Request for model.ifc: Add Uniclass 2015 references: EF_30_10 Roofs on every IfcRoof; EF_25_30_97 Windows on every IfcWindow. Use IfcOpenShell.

First a look at what the model holds.

```python
import ifcopenshell

model = ifcopenshell.open("model.ifc")
print(model.schema)
print("classifications:", [c.Name for c in model.by_type("IfcClassification")])
for ifc_class in ("IfcDoor", "IfcRoof", "IfcStair", "IfcWall", "IfcWindow"):
    print(ifc_class, len(model.by_type(ifc_class)))
```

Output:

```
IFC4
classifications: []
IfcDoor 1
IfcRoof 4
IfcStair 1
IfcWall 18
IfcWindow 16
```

```python
import ifcopenshell
import ifcopenshell.api.classification

model = ifcopenshell.open("model.ifc")

system = ifcopenshell.api.classification.add_classification(model, classification="Uniclass 2015")

codes = {
    "IfcRoof": ("EF_30_10", "Roofs"),
    "IfcWindow": ("EF_25_30_97", "Windows"),
}
for ifc_class, (code, name) in codes.items():
    products = model.by_type(ifc_class)
    ifcopenshell.api.classification.add_reference(
        model, products=products, classification=system, identification=code, name=name
    )
    print(code, len(products))

model.write("model-out.ifc")
```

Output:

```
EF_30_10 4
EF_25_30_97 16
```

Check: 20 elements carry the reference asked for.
